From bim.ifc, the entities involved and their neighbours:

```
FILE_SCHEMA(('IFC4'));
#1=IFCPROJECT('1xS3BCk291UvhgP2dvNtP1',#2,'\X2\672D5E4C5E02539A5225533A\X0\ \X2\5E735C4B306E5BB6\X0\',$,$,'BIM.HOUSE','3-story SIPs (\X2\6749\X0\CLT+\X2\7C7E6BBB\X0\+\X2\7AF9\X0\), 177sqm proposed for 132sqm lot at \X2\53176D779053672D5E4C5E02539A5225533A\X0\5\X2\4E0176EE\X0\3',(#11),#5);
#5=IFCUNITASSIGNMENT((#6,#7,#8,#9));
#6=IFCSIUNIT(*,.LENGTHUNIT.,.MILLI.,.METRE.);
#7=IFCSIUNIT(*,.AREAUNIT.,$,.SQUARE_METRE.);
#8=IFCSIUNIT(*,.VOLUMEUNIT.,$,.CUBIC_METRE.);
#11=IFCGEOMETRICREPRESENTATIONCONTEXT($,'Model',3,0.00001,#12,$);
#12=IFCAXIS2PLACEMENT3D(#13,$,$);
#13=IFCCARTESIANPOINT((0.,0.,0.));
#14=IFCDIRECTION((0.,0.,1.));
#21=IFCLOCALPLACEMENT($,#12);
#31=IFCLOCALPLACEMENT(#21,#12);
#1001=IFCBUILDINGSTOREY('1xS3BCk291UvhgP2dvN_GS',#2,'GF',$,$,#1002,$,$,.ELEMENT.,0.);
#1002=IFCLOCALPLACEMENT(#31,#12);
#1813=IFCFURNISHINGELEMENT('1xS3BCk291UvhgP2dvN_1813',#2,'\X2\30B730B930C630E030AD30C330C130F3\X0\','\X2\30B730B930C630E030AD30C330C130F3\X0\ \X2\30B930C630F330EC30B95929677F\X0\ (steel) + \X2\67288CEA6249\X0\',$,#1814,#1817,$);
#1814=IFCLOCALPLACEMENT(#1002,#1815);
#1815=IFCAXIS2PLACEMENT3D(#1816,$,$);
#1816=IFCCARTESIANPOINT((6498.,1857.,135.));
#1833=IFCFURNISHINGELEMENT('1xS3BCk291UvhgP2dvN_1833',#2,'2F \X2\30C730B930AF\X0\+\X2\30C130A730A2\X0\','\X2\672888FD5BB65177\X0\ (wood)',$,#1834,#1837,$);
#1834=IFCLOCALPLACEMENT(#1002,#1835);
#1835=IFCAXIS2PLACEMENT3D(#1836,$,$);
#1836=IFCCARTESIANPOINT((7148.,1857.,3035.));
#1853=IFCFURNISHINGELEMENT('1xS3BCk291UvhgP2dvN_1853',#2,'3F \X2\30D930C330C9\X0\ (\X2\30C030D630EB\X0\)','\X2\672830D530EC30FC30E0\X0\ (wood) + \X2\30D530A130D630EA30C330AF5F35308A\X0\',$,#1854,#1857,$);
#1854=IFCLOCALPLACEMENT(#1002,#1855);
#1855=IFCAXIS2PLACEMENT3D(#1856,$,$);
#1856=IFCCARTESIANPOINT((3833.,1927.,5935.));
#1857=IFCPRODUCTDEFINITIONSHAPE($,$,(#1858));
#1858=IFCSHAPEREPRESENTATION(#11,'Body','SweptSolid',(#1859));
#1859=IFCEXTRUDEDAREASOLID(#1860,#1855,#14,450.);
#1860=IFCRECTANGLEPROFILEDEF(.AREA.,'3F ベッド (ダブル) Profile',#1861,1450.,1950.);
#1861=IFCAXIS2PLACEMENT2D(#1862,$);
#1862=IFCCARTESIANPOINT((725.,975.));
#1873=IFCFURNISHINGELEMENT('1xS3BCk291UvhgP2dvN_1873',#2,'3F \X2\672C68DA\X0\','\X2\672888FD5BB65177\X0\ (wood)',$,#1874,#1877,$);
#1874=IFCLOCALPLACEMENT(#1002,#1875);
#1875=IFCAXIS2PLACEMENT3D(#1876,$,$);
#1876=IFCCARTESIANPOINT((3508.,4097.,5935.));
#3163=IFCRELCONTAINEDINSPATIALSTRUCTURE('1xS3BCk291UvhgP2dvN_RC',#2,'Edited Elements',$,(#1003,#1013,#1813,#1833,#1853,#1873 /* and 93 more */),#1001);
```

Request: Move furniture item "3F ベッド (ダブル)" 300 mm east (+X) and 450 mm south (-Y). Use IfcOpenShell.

```python
import ifcopenshell
import ifcopenshell.api.geometry
import ifcopenshell.util.placement
import ifcopenshell.util.unit

model = ifcopenshell.open("bim.ifc")
unit_scale = ifcopenshell.util.unit.calculate_unit_scale(model)

item = model.by_guid("1xS3BCk291UvhgP2dvN_1853")
matrix = ifcopenshell.util.placement.get_local_placement(item.ObjectPlacement)
matrix[0, 3] += 0.3 / unit_scale
matrix[1, 3] -= 0.45 / unit_scale
ifcopenshell.api.geometry.edit_object_placement(model, product=item, matrix=matrix, is_si=False)

print(ifcopenshell.util.placement.get_local_placement(item.ObjectPlacement).round(3) + 0.0)

model.write("bim_v2.ifc")
```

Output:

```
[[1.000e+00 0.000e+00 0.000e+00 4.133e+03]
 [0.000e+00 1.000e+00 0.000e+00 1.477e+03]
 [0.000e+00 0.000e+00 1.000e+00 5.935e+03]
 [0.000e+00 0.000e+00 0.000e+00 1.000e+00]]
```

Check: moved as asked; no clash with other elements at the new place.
